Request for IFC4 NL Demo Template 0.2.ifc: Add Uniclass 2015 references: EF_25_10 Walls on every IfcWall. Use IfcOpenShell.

First a look at what the model holds.

```python
import ifcopenshell

model = ifcopenshell.open("IFC4 NL Demo Template 0.2.ifc")
print(model.schema)
print("classifications:", [c.Name for c in model.by_type("IfcClassification")])
for ifc_class in ("IfcDoor", "IfcRoof", "IfcStair", "IfcWall", "IfcWindow"):
    print(ifc_class, len(model.by_type(ifc_class)))
```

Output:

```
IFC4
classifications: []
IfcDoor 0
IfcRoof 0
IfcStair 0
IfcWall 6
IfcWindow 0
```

```python
import ifcopenshell
import ifcopenshell.api.classification

model = ifcopenshell.open("IFC4 NL Demo Template 0.2.ifc")

system = ifcopenshell.api.classification.add_classification(model, classification="Uniclass 2015")

codes = {
    "IfcWall": ("EF_25_10", "Walls"),
}
for ifc_class, (code, name) in codes.items():
    products = model.by_type(ifc_class)
    ifcopenshell.api.classification.add_reference(
        model, products=products, classification=system, identification=code, name=name
    )
    print(code, len(products))

model.write("IFC4 NL Demo Template 0.2_updated.ifc")
```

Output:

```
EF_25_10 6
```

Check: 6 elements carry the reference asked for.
